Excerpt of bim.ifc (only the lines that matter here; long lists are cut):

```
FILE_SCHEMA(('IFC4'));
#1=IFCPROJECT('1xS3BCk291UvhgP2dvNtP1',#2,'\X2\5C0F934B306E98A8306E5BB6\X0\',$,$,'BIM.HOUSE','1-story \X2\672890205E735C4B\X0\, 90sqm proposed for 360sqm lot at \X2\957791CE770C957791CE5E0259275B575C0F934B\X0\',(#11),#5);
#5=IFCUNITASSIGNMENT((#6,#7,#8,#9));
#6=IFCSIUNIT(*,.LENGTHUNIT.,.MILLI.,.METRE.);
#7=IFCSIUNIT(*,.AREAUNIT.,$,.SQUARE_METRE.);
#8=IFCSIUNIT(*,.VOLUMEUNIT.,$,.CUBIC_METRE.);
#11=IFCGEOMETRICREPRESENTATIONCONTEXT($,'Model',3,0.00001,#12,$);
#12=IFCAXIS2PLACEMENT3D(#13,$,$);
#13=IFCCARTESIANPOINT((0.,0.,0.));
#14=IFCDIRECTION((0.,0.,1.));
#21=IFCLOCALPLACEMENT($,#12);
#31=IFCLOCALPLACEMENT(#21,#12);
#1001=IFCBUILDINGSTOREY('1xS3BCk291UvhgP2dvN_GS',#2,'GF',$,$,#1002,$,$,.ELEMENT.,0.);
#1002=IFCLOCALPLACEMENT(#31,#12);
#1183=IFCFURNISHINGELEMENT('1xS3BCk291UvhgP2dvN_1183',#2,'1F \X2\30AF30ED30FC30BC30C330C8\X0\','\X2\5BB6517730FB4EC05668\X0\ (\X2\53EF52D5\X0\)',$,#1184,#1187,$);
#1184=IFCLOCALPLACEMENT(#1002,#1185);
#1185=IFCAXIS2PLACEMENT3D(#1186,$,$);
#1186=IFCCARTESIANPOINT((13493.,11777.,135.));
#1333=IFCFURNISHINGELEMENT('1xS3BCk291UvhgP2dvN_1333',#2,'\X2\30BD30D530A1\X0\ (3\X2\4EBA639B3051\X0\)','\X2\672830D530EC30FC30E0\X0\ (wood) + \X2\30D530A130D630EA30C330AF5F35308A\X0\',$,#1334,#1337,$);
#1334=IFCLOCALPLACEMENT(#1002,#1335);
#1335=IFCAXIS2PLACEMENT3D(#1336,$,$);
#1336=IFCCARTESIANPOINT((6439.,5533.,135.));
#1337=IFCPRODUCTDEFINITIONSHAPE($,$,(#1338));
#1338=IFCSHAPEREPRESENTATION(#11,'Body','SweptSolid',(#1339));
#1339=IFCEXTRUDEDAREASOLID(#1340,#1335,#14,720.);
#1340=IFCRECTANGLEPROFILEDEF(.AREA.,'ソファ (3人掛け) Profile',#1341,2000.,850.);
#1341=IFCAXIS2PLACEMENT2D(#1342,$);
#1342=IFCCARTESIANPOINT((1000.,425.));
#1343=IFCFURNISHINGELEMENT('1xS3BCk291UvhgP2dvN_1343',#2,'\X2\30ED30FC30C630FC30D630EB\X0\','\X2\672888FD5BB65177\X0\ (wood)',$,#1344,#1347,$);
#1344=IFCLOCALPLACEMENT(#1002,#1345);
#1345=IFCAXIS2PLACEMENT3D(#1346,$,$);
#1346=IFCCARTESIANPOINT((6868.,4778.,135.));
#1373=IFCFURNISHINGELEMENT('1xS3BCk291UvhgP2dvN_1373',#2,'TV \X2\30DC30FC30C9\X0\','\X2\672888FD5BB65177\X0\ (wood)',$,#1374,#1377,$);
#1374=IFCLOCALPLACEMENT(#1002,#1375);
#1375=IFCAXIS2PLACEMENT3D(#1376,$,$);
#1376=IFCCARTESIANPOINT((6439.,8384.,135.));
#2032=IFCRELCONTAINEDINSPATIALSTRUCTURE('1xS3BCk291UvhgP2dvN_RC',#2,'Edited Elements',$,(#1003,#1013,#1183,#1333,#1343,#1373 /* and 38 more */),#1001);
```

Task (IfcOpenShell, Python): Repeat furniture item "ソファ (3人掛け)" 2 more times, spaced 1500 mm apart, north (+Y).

```python
import numpy as np
import ifcopenshell
import ifcopenshell.api.geometry
import ifcopenshell.api.root
import ifcopenshell.util.element
import ifcopenshell.util.placement

model = ifcopenshell.open("bim.ifc")


def reuse_history(source, copy):
    """copy_class also copies each property set's owner history, people and application; keep the originals."""
    for rel in copy.IsDefinedBy:
        if rel.is_a("IfcRelDefinesByProperties") and (history := rel.RelatingPropertyDefinition.OwnerHistory):
            rel.RelatingPropertyDefinition.OwnerHistory = source.OwnerHistory
            ifcopenshell.util.element.remove_deep2(model, history)


source = model.by_id(1333)
base = ifcopenshell.util.placement.get_local_placement(source.ObjectPlacement)
step = np.array([0.0, 1.0, 0.0]) * 1500.0

for i in range(1, 3):
    copy = ifcopenshell.api.root.copy_class(model, product=source)
    copy.Representation = ifcopenshell.util.element.copy_deep(
        model, source.Representation, exclude=["IfcGeometricRepresentationContext", "IfcRepresentationMap"]
    )
    reuse_history(source, copy)
    matrix = base.copy()
    matrix[:3, 3] += i * step
    print("added at", matrix[:3, 3].round(3) + 0.0)
    ifcopenshell.api.geometry.edit_object_placement(model, product=copy, matrix=matrix, is_si=False)

model.write("bim_updated.ifc")
```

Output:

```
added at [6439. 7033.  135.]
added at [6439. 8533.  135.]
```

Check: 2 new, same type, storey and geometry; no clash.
